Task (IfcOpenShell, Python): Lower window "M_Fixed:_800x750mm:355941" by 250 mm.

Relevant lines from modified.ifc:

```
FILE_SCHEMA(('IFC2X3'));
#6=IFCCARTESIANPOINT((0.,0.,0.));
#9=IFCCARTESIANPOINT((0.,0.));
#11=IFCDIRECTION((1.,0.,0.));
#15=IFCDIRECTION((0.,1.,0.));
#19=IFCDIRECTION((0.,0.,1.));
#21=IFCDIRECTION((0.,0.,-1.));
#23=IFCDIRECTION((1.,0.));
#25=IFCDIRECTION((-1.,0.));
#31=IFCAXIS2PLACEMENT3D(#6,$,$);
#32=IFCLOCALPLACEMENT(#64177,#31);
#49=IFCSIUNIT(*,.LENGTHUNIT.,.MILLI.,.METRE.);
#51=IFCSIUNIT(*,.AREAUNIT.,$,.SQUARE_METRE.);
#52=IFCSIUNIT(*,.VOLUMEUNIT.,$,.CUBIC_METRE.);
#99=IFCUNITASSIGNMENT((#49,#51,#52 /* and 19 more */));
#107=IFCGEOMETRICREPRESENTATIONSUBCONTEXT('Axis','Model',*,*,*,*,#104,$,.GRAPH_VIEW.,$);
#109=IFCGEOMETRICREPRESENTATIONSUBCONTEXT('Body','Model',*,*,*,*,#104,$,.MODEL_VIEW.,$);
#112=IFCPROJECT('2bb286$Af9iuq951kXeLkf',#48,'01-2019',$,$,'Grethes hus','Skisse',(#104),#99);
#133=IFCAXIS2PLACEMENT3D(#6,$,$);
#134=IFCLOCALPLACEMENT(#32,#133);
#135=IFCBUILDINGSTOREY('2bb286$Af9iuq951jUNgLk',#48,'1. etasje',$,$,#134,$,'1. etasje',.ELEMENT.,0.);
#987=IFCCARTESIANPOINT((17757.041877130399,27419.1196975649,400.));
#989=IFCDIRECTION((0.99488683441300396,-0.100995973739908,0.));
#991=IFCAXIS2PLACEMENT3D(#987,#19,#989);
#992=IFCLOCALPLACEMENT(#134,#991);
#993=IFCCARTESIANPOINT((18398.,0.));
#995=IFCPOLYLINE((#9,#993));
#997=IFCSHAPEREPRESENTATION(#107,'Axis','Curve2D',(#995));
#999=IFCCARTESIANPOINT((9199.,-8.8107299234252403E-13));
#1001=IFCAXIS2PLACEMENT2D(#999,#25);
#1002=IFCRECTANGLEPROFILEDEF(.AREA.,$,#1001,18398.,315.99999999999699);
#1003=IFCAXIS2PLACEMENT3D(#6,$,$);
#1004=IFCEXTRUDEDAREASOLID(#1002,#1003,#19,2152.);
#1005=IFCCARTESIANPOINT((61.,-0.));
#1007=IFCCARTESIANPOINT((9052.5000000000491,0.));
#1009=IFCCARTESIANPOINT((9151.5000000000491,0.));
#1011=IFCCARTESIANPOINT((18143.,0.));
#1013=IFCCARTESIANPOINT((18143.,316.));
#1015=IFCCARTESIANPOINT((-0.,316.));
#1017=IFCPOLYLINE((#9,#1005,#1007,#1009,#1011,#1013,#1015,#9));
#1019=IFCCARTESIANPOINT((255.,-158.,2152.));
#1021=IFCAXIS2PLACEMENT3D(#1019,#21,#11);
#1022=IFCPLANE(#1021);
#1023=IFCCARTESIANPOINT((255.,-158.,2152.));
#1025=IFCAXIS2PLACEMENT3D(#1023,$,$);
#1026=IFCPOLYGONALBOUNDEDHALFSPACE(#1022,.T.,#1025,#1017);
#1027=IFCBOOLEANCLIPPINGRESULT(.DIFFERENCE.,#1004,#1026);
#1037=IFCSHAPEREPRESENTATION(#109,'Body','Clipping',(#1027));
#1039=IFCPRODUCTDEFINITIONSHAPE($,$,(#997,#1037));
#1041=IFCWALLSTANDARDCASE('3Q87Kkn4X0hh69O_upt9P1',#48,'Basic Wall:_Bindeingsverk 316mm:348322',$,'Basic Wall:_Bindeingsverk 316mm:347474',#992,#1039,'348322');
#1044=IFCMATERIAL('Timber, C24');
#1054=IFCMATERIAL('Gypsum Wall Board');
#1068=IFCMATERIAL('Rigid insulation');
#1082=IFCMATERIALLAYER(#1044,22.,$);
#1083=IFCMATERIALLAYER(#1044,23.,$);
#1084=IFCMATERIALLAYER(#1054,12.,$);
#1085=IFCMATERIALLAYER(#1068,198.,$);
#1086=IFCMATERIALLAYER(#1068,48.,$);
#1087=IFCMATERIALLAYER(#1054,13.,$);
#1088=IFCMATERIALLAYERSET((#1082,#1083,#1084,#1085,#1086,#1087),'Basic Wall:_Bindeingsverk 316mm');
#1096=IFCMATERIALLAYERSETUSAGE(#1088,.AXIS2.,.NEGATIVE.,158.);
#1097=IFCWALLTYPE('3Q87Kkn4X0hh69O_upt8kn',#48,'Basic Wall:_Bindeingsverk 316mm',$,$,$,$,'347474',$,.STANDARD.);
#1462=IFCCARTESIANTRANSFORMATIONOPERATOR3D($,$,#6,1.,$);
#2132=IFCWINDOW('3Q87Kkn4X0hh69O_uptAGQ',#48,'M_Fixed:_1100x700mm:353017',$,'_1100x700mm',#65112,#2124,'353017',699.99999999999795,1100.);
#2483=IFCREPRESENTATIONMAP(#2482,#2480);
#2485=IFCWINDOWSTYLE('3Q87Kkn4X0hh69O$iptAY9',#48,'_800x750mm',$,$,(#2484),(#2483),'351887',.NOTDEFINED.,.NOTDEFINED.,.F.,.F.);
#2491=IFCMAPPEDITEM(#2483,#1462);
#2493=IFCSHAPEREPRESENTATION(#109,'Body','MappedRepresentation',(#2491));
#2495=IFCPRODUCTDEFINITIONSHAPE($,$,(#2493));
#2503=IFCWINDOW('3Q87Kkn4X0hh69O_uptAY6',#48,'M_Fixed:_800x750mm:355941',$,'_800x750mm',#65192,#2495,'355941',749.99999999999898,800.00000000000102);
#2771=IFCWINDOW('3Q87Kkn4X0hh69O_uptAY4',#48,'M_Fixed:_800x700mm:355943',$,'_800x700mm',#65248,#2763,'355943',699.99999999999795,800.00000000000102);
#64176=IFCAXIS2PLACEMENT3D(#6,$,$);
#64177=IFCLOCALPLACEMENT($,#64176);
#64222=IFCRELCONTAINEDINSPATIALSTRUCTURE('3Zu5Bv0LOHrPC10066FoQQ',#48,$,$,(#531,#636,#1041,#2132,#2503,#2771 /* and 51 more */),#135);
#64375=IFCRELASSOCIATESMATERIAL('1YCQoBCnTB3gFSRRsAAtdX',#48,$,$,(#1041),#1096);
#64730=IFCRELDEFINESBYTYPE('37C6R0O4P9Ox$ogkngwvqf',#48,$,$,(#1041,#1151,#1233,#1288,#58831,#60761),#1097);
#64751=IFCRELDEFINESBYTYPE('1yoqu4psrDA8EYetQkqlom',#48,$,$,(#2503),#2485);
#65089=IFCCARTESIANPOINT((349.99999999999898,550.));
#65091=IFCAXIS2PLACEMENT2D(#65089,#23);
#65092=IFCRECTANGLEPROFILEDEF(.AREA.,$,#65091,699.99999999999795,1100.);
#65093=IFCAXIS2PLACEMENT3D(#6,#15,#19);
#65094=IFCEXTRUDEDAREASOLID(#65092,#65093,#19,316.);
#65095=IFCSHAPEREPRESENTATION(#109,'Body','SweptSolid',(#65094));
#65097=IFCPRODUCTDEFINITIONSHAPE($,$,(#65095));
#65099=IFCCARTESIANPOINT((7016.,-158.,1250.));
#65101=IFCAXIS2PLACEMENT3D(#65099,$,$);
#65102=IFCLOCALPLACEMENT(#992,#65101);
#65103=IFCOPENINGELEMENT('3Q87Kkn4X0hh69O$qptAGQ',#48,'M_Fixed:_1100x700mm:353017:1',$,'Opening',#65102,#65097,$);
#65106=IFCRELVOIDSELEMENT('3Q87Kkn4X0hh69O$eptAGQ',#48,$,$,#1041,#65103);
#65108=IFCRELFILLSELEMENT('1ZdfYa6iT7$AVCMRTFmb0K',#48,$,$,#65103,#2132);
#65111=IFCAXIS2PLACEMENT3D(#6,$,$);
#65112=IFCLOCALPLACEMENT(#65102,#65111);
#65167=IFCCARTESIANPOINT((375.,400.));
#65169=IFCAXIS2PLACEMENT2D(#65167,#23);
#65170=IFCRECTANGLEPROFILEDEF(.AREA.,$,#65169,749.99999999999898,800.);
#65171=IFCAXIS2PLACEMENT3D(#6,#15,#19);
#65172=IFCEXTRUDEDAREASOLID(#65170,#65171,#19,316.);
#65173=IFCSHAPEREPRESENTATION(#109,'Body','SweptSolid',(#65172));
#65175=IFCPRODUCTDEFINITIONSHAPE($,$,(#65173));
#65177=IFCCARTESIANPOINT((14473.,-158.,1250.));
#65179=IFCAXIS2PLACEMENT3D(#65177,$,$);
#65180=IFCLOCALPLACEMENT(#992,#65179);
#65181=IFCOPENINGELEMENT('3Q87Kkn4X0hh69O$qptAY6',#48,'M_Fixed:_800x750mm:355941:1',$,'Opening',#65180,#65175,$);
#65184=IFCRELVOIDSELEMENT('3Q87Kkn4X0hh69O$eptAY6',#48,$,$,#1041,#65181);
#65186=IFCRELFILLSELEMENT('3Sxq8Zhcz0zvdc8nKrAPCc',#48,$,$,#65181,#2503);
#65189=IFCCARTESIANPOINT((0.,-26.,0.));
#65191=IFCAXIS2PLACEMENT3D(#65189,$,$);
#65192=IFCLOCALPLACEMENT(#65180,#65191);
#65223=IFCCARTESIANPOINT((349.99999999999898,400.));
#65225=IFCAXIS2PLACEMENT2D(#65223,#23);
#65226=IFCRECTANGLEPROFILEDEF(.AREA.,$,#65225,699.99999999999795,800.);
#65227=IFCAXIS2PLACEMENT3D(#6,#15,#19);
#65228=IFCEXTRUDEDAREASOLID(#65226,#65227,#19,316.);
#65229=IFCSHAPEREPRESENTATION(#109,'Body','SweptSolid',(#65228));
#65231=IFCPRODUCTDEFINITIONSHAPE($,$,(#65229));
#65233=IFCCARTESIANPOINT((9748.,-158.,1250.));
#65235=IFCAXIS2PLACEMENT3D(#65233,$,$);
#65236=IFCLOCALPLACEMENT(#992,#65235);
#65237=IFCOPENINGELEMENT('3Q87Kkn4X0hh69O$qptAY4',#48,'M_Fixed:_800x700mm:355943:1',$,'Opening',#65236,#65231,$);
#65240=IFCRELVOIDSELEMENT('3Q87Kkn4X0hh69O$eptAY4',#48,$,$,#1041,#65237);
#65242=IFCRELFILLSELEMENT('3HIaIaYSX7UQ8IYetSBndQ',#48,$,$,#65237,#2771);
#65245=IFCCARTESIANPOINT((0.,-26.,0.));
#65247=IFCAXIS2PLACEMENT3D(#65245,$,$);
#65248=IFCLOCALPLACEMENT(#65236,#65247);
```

```python
import numpy as np
import ifcopenshell
import ifcopenshell.api.geometry
import ifcopenshell.util.placement
import ifcopenshell.util.unit

model = ifcopenshell.open("modified.ifc")
unit_scale = ifcopenshell.util.unit.calculate_unit_scale(model)

window = model.by_guid("3Q87Kkn4X0hh69O_uptAY6")
opening = window.FillsVoids[0].RelatingOpeningElement
dz = -250.0

shift = np.array([0.0, 0.0, dz])
# The window is placed relative to its opening, so it follows when the opening moves.
matrix = ifcopenshell.util.placement.get_local_placement(opening.ObjectPlacement)
matrix[:3, 3] += shift
ifcopenshell.api.geometry.edit_object_placement(
    model, product=opening, matrix=matrix, is_si=False, should_transform_children=True
)

print(f"moved by {dz * unit_scale:+.3f} m")

model.write("modified_updated.ifc")
```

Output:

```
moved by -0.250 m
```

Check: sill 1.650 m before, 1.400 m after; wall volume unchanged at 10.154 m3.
